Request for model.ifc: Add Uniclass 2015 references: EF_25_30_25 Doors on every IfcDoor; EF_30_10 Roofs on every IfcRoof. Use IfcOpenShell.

First a look at what the model holds.

```python
import ifcopenshell

model = ifcopenshell.open("model.ifc")
print(model.schema)
print("classifications:", [c.Name for c in model.by_type("IfcClassification")])
for ifc_class in ("IfcDoor", "IfcRoof", "IfcStair", "IfcWall", "IfcWindow"):
    print(ifc_class, len(model.by_type(ifc_class)))
```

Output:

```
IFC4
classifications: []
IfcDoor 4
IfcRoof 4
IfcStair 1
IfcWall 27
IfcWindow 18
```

```python
import ifcopenshell
import ifcopenshell.api.classification

model = ifcopenshell.open("model.ifc")

system = ifcopenshell.api.classification.add_classification(model, classification="Uniclass 2015")

codes = {
    "IfcDoor": ("EF_25_30_25", "Doors"),
    "IfcRoof": ("EF_30_10", "Roofs"),
}
for ifc_class, (code, name) in codes.items():
    products = model.by_type(ifc_class)
    ifcopenshell.api.classification.add_reference(
        model, products=products, classification=system, identification=code, name=name
    )
    print(code, len(products))

model.write("model_rev.ifc")
```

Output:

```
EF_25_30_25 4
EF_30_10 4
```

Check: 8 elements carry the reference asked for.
